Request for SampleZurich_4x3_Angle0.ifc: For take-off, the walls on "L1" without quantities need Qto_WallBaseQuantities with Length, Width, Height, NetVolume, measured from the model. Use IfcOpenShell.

First a look at what the model holds.

```python
import ifcopenshell
import ifcopenshell.util.element
import ifcopenshell.util.unit

model = ifcopenshell.open("SampleZurich_4x3_Angle0.ifc")
print(model.schema)
for unit_type in ("LENGTHUNIT", "AREAUNIT", "VOLUMEUNIT"):
    print(unit_type, ifcopenshell.util.unit.calculate_unit_scale(model, unit_type))
storey = next(s for s in model.by_type("IfcBuildingStorey") if s.Name == "L1")
walls = [e for e in ifcopenshell.util.element.get_decomposition(storey) if e.is_a("IfcWall")]
for e in sorted(walls, key=lambda e: e.id()):
    print(e.id(), e.is_a(), e.Name, list(ifcopenshell.util.element.get_psets(e, qtos_only=True)), sep=" | ")
```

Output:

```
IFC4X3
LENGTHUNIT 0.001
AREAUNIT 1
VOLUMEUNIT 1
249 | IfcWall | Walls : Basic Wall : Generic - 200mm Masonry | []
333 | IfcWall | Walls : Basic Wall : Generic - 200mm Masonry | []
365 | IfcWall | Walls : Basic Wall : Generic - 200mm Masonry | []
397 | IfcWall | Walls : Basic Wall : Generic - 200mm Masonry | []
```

```python
import ifcopenshell
import ifcopenshell.api.pset
import ifcopenshell.geom
import ifcopenshell.util.element
import ifcopenshell.util.shape
import ifcopenshell.util.unit

model = ifcopenshell.open("SampleZurich_4x3_Angle0.ifc")
unit_scale = ifcopenshell.util.unit.calculate_unit_scale(model)
volume_scale = ifcopenshell.util.unit.calculate_unit_scale(model, "VOLUMEUNIT")
settings = ifcopenshell.geom.settings()

storey = next(s for s in model.by_type("IfcBuildingStorey") if s.Name == "L1")
walls = [e for e in ifcopenshell.util.element.get_decomposition(storey) if e.is_a("IfcWall")]

for e in sorted(walls, key=lambda e: e.id()):
    if ifcopenshell.util.element.get_psets(e, qtos_only=True, should_inherit=False):
        continue
    # Geometry comes back in metres, in the element's own axes.
    shape = ifcopenshell.geom.create_shape(settings, e)
    values = {
        "Length": ifcopenshell.util.shape.get_x(shape.geometry) / unit_scale,
        "Width": ifcopenshell.util.shape.get_y(shape.geometry) / unit_scale,
        "Height": ifcopenshell.util.shape.get_z(shape.geometry) / unit_scale,
        "NetVolume": ifcopenshell.util.shape.get_volume(shape.geometry) / volume_scale,
    }
    qto = ifcopenshell.api.pset.add_qto(model, product=e, name="Qto_WallBaseQuantities")
    ifcopenshell.api.pset.edit_qto(model, qto=qto, properties=values)
    print(e.id(), {k: round(v, 3) for k, v in values.items()})

model.write("SampleZurich_4x3_Angle0_rev.ifc")
```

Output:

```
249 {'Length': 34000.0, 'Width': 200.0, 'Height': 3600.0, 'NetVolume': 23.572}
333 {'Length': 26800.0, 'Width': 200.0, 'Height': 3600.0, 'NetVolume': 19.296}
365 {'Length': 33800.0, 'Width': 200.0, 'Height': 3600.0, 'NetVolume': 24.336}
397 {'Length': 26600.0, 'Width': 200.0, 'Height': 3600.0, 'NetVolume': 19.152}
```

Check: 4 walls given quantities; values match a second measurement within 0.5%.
